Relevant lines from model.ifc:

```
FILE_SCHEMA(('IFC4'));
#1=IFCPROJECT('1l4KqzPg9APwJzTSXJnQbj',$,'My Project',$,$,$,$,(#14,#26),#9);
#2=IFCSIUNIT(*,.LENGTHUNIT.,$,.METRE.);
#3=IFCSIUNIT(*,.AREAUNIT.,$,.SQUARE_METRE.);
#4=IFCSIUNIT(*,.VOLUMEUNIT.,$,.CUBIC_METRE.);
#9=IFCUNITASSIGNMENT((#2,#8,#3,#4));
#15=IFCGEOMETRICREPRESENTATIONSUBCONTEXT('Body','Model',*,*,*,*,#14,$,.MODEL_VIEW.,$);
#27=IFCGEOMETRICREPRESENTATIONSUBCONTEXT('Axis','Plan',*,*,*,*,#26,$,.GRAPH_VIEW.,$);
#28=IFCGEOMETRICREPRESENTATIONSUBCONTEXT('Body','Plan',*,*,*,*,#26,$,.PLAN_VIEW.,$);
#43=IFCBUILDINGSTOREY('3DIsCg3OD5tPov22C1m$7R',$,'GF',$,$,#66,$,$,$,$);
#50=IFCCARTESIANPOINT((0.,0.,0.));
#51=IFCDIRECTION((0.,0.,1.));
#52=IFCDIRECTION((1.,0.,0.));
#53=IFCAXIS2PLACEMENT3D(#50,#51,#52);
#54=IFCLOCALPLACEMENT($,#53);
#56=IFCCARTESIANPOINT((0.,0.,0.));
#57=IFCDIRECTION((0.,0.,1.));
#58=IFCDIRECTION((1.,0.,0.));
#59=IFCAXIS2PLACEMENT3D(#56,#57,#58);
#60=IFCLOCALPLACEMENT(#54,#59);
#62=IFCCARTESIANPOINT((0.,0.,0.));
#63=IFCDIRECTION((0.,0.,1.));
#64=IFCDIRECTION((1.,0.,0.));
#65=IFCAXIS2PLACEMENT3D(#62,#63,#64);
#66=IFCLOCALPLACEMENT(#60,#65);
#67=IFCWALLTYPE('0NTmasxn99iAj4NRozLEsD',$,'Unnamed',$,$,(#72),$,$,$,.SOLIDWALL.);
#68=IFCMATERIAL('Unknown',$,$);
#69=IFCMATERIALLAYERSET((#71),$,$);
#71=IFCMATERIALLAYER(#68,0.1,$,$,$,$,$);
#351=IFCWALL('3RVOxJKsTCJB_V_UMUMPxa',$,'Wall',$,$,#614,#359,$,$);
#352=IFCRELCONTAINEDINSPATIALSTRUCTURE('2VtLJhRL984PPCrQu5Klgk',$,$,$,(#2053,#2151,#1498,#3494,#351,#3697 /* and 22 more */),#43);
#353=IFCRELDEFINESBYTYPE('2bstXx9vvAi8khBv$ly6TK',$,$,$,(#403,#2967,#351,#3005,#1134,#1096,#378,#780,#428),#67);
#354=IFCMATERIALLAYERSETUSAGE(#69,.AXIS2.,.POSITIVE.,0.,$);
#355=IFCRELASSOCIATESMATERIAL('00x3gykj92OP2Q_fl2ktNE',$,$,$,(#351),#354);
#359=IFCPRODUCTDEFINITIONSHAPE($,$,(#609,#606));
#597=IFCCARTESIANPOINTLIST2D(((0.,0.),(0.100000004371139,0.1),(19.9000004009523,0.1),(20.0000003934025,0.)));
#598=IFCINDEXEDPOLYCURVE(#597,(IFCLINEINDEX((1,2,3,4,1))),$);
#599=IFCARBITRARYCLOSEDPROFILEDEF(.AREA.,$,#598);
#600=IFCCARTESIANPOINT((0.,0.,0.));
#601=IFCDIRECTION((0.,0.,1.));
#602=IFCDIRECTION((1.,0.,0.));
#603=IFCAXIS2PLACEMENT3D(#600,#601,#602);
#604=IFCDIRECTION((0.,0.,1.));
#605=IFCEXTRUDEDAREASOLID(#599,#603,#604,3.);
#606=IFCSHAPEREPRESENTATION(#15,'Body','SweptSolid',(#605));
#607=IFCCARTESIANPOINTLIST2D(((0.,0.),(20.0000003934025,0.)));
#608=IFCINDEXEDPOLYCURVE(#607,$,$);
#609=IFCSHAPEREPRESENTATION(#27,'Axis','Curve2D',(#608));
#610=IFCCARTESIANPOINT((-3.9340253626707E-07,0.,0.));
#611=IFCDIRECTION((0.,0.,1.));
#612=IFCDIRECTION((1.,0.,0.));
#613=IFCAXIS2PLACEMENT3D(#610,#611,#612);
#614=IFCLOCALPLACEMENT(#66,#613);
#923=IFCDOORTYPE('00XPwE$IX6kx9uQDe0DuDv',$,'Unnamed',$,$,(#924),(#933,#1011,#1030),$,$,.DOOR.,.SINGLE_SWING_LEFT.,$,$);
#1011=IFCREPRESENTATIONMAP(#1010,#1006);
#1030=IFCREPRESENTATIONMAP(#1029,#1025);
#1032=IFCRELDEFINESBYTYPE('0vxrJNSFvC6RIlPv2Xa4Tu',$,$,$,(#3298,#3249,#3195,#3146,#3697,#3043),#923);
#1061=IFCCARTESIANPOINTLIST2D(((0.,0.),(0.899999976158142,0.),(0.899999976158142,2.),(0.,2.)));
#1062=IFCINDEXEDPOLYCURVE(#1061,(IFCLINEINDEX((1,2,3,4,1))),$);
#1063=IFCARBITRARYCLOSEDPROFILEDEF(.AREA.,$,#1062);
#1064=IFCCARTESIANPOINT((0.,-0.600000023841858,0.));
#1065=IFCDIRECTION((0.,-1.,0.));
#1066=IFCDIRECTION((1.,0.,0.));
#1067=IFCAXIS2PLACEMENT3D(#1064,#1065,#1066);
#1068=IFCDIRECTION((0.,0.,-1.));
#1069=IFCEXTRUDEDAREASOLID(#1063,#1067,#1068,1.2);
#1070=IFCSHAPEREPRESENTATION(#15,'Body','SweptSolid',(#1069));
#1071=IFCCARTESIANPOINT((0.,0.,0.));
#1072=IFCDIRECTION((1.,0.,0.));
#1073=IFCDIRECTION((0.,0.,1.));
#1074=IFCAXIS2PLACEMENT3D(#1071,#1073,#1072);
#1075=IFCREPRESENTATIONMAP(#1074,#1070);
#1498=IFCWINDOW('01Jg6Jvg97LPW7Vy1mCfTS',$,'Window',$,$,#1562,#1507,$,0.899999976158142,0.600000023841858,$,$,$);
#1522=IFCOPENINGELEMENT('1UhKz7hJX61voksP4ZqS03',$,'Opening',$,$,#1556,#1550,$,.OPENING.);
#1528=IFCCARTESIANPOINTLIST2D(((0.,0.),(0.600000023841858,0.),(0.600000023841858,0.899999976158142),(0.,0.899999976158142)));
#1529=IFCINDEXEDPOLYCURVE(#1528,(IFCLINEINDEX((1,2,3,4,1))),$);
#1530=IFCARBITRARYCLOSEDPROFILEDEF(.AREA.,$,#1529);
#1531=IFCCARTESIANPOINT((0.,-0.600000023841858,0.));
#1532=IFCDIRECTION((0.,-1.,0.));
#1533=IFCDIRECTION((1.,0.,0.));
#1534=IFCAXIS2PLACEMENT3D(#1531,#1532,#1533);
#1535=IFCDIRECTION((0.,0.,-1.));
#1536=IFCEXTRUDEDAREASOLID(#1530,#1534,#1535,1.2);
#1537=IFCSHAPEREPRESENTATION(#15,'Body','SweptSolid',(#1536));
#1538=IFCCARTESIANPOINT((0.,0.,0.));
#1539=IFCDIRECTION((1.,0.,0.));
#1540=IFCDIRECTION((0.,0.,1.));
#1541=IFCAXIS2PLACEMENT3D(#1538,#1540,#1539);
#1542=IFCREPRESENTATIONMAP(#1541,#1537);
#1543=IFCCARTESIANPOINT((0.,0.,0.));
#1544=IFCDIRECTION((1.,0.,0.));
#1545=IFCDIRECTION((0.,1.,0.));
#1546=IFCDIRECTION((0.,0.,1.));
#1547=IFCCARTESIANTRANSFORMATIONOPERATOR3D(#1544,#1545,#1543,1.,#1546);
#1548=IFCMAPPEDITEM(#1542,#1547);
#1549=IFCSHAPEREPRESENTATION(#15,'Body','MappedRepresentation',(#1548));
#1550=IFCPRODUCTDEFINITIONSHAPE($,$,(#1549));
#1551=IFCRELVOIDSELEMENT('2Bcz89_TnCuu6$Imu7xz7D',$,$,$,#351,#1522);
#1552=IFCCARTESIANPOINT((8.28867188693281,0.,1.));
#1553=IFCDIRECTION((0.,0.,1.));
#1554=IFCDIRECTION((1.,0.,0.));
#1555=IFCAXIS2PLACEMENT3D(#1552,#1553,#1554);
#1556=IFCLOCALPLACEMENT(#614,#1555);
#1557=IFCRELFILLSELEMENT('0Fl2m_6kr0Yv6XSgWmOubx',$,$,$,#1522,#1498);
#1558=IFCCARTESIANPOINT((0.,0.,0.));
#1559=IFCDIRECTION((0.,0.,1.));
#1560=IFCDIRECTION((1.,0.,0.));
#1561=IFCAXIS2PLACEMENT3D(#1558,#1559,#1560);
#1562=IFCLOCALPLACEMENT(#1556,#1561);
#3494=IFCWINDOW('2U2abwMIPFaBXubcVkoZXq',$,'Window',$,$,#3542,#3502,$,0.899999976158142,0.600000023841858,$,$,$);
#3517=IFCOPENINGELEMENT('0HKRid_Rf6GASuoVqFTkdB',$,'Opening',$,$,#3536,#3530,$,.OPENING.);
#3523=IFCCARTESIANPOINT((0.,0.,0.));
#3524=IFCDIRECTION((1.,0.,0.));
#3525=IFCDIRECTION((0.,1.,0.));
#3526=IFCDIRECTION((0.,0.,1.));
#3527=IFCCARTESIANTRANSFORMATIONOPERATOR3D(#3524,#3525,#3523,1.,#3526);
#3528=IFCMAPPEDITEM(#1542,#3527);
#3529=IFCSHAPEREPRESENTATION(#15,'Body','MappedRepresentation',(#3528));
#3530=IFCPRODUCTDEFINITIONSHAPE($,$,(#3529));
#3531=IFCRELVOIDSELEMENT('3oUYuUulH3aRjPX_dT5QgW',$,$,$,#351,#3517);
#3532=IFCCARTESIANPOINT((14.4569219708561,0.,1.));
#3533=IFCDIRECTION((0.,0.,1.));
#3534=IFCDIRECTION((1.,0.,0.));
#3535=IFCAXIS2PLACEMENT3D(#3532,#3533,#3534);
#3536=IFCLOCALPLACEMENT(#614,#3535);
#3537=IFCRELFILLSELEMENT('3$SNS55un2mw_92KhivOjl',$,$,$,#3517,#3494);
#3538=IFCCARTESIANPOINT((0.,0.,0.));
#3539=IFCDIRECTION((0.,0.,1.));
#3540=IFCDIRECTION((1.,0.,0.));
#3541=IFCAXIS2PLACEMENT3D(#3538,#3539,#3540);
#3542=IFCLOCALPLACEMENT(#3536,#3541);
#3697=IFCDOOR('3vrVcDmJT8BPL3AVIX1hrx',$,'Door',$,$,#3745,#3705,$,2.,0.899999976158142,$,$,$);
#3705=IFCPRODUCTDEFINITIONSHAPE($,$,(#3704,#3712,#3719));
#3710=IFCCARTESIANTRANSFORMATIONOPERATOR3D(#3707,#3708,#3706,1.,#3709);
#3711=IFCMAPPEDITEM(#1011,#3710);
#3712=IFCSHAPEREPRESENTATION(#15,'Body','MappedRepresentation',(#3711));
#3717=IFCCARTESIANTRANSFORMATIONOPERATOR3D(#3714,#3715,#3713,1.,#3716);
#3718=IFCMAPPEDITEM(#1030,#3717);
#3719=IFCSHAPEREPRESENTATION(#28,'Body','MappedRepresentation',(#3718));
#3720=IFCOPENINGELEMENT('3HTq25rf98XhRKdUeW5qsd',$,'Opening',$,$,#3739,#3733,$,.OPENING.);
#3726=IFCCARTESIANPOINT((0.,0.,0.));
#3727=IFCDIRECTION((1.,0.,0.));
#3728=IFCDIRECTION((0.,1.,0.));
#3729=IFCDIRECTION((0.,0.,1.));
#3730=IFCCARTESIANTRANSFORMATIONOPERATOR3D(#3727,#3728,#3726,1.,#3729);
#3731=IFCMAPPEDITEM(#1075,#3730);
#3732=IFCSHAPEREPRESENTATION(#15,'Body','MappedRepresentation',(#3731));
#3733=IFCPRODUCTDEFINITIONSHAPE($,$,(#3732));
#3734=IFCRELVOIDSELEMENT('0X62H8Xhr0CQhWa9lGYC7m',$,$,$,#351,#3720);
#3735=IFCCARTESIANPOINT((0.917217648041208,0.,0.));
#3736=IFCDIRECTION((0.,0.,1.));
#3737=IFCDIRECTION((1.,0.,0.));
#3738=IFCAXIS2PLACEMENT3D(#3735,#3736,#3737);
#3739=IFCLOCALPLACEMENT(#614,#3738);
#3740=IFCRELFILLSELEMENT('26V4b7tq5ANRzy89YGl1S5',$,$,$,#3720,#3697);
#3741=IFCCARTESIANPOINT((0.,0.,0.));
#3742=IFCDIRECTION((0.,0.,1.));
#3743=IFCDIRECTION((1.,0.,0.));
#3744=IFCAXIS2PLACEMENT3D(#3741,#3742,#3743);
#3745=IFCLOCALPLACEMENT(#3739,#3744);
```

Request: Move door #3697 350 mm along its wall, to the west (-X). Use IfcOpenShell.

```python
import ifcopenshell
import ifcopenshell.api.geometry
import ifcopenshell.util.placement

model = ifcopenshell.open("model.ifc")

door = model.by_guid("3vrVcDmJT8BPL3AVIX1hrx")
opening = door.FillsVoids[0].RelatingOpeningElement
wall = opening.VoidsElements[0].RelatingBuildingElement

wall_matrix = ifcopenshell.util.placement.get_local_placement(wall.ObjectPlacement)
shift = wall_matrix[:3, 0] * -0.35
before = ifcopenshell.util.placement.get_local_placement(door.ObjectPlacement)[:3, 3].copy()

# The door is placed relative to its opening, so it follows when the opening moves.
matrix = ifcopenshell.util.placement.get_local_placement(opening.ObjectPlacement)
matrix[:3, 3] += shift
ifcopenshell.api.geometry.edit_object_placement(
    model, product=opening, matrix=matrix, is_si=False, should_transform_children=True
)

after = ifcopenshell.util.placement.get_local_placement(door.ObjectPlacement)[:3, 3]
print("door moved by", (after - before).round(3) + 0.0)

model.write("model_rev.ifc")
```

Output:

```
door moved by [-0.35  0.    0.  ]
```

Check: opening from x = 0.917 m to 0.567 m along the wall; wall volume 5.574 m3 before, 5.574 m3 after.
